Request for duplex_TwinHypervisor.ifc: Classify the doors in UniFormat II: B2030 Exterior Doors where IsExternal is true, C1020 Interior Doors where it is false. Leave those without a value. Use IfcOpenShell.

First a look at what the model holds.

```python
import ifcopenshell
import ifcopenshell.util.element

model = ifcopenshell.open("duplex_TwinHypervisor.ifc")
print(model.schema)
print("classifications:", [c.Name for c in model.by_type("IfcClassification")])
values = [ifcopenshell.util.element.get_pset(e, "Pset_DoorCommon", "IsExternal") for e in model.by_type("IfcDoor")]
for value in (True, False, None):
    print("IsExternal", value, values.count(value))
```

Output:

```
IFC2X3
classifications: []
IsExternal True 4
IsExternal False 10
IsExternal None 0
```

```python
import ifcopenshell
import ifcopenshell.api.classification
import ifcopenshell.util.element

model = ifcopenshell.open("duplex_TwinHypervisor.ifc")

# IFC2X3 requires Source and Edition and has no link from the project to the system.
system = model.create_entity("IfcClassification", Source="ASTM", Edition="E1557", Name="UniFormat II")

doors = model.by_type("IfcDoor")
external = {e: ifcopenshell.util.element.get_pset(e, "Pset_DoorCommon", "IsExternal") for e in doors}
for flag, code, name in ((True, "B2030", "Exterior Doors"), (False, "C1020", "Interior Doors")):
    products = [e for e in doors if external[e] is flag]
    ifcopenshell.api.classification.add_reference(
        model, products=products, classification=system, identification=code, name=name
    )
    print(code, len(products))

model.write("duplex_TwinHypervisor_v2.ifc")
```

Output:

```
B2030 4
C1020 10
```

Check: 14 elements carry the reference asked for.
